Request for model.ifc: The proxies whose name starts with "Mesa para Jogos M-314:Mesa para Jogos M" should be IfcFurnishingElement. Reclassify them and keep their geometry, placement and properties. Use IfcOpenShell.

First a look at what the model holds.

```python
import re

import ifcopenshell

model = ifcopenshell.open("model.ifc")
print(model.schema)
seen = {}
for e in model.by_type("IfcBuildingElementProxy"):
    name = re.sub(r":\d+(:\d+)?$", "", e.Name or "")  # drop the element id that some exporters append
    seen[name] = seen.get(name, 0) + 1
for name, count in sorted(seen.items()):
    print(count, "x", name)
```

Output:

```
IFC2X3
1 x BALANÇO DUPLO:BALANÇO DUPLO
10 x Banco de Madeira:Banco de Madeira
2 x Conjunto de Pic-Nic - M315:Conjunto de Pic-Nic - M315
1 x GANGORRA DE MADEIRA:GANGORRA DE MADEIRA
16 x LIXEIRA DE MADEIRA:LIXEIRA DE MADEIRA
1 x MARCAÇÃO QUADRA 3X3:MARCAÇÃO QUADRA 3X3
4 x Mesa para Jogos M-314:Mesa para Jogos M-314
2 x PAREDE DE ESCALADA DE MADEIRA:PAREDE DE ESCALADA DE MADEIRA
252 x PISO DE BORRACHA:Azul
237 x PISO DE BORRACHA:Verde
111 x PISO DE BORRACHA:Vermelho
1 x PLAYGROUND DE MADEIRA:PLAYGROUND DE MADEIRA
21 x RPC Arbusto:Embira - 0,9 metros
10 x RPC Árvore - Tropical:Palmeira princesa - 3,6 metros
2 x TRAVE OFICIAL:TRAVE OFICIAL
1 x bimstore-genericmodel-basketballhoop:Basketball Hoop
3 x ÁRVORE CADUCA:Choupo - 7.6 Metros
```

```python
import ifcopenshell
import ifcopenshell.api.root

model = ifcopenshell.open("model.ifc")

proxies = [e.id() for e in model.by_type("IfcBuildingElementProxy") if (e.Name or "").startswith("Mesa para Jogos M-314:Mesa para Jogos M")]
for step_id in proxies:
    proxy = model.by_id(step_id)
    # Reclassifying a typed element also reclassifies its type and the type's other occurrences.
    if proxy.is_a("IfcBuildingElementProxy"):
        ifcopenshell.api.root.reassign_class(model, product=proxy, ifc_class="IfcFurnishingElement")

print(sum(model.by_id(i).is_a("IfcFurnishingElement") for i in proxies), "reclassified")

model.write("model_edited.ifc")
```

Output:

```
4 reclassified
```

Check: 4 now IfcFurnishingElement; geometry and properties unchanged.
